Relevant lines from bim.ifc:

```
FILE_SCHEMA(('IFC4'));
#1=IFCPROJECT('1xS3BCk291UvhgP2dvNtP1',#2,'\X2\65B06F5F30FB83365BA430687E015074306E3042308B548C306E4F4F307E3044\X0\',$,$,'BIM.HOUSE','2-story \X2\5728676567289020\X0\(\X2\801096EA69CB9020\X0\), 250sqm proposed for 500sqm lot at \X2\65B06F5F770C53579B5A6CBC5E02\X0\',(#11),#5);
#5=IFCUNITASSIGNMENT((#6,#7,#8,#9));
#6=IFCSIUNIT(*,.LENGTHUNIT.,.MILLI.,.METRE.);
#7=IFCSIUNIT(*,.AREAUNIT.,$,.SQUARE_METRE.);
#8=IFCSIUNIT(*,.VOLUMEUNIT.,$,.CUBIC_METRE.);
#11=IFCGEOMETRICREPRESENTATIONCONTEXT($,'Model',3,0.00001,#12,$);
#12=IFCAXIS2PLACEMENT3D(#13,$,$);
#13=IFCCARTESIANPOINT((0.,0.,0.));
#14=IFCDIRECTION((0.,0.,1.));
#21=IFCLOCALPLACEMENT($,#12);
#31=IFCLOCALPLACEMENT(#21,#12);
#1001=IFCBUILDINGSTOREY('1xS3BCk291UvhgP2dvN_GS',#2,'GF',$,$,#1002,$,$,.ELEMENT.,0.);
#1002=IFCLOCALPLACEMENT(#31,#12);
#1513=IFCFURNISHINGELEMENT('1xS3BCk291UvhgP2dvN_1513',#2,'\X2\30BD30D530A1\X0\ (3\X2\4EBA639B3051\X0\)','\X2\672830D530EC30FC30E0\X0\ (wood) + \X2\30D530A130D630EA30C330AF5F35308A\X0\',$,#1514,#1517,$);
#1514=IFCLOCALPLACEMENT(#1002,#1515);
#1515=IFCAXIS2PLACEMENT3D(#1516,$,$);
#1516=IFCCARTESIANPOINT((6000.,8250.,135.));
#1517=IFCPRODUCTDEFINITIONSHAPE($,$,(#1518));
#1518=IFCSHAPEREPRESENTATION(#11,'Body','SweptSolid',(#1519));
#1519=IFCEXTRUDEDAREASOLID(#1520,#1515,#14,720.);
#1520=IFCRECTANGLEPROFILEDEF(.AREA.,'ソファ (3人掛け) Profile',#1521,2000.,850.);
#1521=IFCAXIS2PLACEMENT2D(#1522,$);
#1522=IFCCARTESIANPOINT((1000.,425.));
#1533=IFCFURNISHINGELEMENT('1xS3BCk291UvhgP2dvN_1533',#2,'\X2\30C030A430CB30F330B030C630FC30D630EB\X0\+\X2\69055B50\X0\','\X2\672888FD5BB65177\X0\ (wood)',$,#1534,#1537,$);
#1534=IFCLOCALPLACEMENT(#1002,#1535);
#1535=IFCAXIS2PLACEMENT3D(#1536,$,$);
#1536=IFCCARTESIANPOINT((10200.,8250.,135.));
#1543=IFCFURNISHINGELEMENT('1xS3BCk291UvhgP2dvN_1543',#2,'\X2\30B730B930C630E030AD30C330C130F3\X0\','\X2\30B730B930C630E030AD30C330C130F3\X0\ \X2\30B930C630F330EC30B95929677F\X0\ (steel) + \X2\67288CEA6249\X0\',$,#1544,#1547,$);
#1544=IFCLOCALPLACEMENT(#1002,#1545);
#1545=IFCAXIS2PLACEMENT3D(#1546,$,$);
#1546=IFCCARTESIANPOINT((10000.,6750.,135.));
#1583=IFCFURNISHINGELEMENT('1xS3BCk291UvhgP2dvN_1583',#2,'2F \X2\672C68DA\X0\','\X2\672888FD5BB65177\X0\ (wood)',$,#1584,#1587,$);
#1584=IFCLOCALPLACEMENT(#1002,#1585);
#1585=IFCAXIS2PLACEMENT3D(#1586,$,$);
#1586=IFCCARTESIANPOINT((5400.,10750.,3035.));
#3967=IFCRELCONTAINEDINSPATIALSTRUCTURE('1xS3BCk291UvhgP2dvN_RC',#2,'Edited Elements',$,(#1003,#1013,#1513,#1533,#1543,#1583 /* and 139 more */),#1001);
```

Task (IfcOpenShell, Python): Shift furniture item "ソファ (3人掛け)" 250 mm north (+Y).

```python
import ifcopenshell
import ifcopenshell.api.geometry
import ifcopenshell.util.placement
import ifcopenshell.util.unit

model = ifcopenshell.open("bim.ifc")
unit_scale = ifcopenshell.util.unit.calculate_unit_scale(model)

item = model.by_guid("1xS3BCk291UvhgP2dvN_1513")
matrix = ifcopenshell.util.placement.get_local_placement(item.ObjectPlacement)
matrix[1, 3] += 0.25 / unit_scale
ifcopenshell.api.geometry.edit_object_placement(model, product=item, matrix=matrix, is_si=False)

print(ifcopenshell.util.placement.get_local_placement(item.ObjectPlacement).round(3) + 0.0)

model.write("bim_v2.ifc")
```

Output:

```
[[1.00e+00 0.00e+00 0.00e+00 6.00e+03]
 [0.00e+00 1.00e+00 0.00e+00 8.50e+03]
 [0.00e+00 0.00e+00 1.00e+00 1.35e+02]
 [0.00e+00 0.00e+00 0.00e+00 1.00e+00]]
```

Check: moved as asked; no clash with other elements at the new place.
